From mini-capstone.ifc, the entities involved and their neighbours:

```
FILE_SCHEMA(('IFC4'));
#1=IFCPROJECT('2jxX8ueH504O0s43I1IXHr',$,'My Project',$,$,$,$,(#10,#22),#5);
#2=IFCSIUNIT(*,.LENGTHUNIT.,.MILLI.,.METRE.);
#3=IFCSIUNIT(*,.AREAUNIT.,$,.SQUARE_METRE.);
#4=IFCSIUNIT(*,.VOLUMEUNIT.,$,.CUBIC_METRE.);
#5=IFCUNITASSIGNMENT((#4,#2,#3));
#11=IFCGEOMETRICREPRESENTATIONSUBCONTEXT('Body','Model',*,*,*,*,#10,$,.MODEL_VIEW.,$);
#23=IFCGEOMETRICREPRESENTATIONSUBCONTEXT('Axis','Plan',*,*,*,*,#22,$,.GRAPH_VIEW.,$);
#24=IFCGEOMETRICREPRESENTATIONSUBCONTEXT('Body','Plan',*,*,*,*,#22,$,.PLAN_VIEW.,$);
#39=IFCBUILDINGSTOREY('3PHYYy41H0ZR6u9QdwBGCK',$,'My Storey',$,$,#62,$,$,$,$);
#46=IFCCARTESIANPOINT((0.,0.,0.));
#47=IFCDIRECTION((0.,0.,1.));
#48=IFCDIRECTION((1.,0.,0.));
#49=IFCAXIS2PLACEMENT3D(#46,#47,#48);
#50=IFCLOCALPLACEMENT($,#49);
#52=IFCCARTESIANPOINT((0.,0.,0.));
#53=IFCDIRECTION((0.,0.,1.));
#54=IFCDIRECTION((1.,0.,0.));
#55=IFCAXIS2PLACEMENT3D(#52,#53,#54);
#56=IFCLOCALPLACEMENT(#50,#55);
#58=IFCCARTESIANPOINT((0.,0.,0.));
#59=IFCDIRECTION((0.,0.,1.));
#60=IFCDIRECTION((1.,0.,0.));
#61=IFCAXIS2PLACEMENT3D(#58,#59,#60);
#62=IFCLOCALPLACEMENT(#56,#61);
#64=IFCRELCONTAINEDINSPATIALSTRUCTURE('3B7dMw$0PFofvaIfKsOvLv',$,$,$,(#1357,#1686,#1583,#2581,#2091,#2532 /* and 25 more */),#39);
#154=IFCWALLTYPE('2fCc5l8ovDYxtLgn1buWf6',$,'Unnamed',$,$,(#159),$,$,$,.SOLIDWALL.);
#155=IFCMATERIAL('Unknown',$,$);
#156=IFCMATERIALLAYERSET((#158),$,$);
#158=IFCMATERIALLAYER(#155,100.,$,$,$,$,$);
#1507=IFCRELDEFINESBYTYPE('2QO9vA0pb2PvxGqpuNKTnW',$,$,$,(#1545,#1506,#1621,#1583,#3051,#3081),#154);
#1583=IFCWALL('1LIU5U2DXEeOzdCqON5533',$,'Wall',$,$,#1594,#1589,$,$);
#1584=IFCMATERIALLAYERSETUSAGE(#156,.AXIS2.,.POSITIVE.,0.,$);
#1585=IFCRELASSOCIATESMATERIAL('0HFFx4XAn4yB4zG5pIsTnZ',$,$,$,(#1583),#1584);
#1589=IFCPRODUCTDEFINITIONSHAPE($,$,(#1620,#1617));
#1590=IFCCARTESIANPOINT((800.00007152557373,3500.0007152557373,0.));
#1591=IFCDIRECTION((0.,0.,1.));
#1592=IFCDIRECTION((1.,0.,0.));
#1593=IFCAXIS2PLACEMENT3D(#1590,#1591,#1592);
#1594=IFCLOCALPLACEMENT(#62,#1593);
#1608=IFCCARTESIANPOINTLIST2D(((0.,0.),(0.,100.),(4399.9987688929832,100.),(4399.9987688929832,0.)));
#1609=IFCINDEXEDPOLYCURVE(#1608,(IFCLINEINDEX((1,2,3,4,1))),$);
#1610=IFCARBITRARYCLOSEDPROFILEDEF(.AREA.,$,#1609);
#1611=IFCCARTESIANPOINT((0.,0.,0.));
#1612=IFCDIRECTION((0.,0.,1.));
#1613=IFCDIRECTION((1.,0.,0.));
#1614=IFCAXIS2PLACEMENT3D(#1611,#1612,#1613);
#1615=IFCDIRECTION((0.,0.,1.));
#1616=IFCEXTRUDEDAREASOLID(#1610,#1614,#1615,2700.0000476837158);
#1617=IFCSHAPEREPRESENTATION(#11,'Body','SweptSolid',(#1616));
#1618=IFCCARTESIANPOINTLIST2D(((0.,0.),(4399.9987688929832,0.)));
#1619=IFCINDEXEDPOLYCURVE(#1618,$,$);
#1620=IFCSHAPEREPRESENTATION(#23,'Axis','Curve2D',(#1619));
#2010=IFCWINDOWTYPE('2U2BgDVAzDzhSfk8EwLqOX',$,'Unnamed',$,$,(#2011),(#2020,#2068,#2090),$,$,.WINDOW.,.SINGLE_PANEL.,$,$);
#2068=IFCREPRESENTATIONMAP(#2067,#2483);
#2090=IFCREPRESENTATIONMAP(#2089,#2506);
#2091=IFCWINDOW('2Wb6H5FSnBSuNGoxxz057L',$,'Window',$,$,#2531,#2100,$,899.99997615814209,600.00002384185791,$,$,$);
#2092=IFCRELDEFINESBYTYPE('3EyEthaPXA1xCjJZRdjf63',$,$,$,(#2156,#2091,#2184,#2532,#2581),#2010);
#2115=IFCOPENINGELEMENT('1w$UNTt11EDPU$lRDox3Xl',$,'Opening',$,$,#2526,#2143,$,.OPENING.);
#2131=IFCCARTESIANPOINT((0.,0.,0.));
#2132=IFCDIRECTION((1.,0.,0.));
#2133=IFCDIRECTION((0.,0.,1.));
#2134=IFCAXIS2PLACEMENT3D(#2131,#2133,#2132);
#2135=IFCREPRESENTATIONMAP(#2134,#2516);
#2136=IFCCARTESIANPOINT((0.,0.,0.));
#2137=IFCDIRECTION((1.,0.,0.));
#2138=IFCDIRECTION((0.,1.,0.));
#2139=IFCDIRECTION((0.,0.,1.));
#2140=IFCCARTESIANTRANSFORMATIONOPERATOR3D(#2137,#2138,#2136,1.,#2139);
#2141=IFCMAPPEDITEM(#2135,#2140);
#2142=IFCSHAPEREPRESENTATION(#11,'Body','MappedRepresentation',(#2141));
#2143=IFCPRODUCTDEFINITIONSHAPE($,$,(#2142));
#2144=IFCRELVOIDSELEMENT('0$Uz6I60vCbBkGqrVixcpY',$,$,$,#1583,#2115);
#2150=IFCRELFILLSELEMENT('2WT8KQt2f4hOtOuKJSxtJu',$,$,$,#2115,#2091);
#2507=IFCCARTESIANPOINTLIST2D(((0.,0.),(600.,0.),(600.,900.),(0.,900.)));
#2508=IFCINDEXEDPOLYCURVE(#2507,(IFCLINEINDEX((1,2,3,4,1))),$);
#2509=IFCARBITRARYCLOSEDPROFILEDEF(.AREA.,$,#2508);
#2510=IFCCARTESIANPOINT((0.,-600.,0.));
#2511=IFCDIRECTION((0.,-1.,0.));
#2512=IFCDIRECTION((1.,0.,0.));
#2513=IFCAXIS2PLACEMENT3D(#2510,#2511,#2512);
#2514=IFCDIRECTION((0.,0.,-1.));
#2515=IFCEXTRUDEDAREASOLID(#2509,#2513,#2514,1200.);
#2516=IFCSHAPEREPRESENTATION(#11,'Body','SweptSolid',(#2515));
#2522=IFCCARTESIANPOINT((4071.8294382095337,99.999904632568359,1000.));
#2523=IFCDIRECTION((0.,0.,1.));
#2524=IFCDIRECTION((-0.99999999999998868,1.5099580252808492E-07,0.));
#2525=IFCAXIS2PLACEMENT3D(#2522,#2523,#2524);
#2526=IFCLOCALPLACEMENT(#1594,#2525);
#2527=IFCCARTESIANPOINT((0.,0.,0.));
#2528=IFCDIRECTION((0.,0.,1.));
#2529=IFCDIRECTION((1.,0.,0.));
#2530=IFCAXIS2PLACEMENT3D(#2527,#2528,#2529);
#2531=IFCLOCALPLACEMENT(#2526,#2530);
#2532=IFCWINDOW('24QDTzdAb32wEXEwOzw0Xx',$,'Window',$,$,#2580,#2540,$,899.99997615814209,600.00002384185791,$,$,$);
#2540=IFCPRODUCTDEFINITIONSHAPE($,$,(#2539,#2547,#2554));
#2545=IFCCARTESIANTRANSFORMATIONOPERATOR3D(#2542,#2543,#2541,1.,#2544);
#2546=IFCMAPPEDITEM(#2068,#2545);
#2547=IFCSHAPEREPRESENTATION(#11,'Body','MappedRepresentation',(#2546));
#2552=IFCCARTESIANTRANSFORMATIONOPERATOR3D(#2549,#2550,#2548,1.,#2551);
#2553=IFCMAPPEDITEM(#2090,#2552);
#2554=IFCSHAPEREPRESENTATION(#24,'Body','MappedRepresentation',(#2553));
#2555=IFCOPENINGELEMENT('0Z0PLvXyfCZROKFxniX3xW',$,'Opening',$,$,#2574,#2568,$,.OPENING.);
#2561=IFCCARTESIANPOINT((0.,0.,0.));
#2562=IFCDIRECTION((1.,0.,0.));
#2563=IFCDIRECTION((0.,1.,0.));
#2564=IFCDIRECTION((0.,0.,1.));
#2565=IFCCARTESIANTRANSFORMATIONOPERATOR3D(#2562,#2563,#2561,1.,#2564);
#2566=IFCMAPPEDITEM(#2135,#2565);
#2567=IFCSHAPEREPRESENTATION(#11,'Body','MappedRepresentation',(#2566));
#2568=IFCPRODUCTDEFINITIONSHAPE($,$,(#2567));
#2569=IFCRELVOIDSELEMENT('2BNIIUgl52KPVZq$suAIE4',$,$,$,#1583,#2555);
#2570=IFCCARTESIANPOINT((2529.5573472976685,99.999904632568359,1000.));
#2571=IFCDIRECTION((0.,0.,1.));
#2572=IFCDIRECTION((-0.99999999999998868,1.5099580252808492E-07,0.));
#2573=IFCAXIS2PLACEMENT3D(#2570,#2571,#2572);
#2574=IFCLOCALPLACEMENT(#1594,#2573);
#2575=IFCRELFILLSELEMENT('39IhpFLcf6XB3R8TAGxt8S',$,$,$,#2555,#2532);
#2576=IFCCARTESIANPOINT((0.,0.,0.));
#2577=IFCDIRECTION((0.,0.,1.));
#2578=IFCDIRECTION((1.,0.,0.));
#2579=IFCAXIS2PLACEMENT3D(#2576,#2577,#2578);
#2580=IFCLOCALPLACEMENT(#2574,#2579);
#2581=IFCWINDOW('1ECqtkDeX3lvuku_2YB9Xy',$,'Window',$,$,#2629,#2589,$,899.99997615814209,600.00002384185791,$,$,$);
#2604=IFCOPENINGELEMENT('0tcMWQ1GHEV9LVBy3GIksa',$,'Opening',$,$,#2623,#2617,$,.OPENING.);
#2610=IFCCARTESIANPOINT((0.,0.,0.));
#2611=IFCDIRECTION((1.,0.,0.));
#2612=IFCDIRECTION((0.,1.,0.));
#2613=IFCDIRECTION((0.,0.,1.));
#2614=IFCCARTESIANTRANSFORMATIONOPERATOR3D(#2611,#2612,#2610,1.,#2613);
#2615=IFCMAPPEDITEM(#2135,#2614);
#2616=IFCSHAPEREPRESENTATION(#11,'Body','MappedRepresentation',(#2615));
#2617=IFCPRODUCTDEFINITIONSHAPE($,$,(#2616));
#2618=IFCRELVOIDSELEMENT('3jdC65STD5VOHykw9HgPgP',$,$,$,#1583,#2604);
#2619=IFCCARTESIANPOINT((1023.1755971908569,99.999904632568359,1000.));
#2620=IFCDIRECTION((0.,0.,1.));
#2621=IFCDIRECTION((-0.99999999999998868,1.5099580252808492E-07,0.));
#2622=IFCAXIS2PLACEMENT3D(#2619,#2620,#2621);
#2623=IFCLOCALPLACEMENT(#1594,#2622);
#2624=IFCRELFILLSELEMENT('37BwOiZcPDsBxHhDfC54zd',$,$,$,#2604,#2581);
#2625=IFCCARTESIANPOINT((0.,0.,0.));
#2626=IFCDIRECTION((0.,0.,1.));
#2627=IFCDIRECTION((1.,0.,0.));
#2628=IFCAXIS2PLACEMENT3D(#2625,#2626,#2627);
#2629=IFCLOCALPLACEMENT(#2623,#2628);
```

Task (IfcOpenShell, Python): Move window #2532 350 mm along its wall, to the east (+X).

```python
import ifcopenshell
import ifcopenshell.api.geometry
import ifcopenshell.util.placement
import ifcopenshell.util.unit

model = ifcopenshell.open("mini-capstone.ifc")
unit_scale = ifcopenshell.util.unit.calculate_unit_scale(model)

window = model.by_guid("24QDTzdAb32wEXEwOzw0Xx")
opening = window.FillsVoids[0].RelatingOpeningElement
wall = opening.VoidsElements[0].RelatingBuildingElement

wall_matrix = ifcopenshell.util.placement.get_local_placement(wall.ObjectPlacement)
shift = wall_matrix[:3, 0] * 0.35 / unit_scale
before = ifcopenshell.util.placement.get_local_placement(window.ObjectPlacement)[:3, 3].copy()

# The window is placed relative to its opening, so it follows when the opening moves.
matrix = ifcopenshell.util.placement.get_local_placement(opening.ObjectPlacement)
matrix[:3, 3] += shift
ifcopenshell.api.geometry.edit_object_placement(
    model, product=opening, matrix=matrix, is_si=False, should_transform_children=True
)

after = ifcopenshell.util.placement.get_local_placement(window.ObjectPlacement)[:3, 3]
print("window moved by", (after - before).round(3) + 0.0)

model.write("mini-capstone-out.ifc")
```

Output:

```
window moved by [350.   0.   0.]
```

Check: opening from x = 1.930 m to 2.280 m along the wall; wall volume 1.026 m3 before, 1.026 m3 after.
